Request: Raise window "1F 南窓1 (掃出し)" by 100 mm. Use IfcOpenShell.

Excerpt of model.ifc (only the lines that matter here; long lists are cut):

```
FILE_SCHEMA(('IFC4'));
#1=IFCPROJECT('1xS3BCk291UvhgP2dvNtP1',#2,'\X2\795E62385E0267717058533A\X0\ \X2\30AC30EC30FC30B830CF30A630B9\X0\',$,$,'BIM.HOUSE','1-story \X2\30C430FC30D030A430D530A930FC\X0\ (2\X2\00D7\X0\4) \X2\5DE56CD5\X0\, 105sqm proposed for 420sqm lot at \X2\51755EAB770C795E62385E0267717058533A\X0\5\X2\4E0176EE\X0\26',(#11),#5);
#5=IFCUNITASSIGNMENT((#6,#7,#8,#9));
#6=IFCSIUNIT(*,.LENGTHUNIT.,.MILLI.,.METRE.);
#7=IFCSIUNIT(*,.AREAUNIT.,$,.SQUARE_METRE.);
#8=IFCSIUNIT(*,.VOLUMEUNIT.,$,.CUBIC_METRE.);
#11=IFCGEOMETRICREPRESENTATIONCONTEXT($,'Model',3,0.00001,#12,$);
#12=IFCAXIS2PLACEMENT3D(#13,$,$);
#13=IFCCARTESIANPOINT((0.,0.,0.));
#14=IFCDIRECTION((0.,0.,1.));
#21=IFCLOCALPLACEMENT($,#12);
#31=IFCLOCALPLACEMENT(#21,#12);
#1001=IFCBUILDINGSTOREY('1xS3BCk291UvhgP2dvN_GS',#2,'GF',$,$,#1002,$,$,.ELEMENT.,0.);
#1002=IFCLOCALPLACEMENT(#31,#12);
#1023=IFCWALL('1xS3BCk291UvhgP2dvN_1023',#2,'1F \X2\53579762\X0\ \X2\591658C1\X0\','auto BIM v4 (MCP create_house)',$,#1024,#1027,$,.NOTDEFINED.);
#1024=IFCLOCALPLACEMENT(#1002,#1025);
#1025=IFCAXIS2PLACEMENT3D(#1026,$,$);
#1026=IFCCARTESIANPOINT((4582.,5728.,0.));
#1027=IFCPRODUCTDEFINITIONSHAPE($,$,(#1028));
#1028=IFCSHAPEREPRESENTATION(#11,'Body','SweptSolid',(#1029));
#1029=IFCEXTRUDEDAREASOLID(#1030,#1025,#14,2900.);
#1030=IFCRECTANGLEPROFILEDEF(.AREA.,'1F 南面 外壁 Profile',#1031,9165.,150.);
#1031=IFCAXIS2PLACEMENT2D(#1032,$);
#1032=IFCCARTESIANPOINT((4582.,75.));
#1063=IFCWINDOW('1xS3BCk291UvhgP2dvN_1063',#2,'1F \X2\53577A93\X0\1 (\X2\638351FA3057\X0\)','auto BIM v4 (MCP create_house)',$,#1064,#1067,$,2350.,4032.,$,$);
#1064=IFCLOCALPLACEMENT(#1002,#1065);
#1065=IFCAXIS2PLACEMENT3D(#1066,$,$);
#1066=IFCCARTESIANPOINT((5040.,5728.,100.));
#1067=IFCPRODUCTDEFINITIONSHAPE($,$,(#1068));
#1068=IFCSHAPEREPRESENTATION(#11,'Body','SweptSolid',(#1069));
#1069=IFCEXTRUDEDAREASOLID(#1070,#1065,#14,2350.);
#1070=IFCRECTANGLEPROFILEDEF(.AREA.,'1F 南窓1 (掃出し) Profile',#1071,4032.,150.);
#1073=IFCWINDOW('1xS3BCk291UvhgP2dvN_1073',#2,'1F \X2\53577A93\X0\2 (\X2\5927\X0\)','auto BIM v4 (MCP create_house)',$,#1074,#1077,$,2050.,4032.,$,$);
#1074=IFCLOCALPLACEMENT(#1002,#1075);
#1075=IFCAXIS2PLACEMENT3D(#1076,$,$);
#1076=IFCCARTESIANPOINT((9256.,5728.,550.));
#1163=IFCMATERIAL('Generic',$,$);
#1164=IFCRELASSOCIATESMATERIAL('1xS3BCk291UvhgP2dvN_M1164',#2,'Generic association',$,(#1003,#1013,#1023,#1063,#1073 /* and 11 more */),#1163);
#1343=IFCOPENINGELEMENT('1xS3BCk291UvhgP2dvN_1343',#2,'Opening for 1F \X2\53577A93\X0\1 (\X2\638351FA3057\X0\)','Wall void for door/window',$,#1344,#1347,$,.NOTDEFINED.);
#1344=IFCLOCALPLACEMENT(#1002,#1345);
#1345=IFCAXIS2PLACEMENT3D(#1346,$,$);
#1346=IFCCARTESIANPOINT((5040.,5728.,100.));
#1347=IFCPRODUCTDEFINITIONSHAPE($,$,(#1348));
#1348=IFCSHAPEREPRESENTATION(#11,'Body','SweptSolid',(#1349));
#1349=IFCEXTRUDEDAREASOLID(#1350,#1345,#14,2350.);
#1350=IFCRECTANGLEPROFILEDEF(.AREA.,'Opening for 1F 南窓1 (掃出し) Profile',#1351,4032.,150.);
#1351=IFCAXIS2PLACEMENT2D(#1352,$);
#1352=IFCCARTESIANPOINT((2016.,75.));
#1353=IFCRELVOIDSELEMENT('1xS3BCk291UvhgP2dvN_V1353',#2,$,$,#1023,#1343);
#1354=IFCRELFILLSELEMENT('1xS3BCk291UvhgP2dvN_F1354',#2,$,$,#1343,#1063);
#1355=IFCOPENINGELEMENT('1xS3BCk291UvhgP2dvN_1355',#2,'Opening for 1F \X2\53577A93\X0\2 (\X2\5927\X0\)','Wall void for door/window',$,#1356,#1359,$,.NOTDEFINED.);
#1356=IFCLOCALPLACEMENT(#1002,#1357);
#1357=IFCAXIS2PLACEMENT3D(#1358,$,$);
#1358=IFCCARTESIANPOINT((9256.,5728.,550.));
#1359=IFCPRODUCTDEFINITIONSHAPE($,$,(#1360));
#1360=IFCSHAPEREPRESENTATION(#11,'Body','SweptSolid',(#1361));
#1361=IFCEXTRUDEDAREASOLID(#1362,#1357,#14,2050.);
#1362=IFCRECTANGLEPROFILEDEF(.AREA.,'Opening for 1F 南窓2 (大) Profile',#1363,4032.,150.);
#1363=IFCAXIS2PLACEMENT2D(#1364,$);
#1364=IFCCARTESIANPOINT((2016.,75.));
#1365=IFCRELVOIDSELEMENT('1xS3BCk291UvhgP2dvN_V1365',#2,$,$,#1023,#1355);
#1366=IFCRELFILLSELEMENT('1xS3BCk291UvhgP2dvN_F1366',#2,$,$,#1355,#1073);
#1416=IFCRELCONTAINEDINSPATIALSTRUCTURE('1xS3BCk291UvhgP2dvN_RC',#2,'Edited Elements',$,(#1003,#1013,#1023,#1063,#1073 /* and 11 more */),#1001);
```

```python
import numpy as np
import ifcopenshell
import ifcopenshell.api.geometry
import ifcopenshell.util.placement
import ifcopenshell.util.unit

model = ifcopenshell.open("model.ifc")
unit_scale = ifcopenshell.util.unit.calculate_unit_scale(model)

window = model.by_guid("1xS3BCk291UvhgP2dvN_1063")
opening = window.FillsVoids[0].RelatingOpeningElement
dz = 0.1 / unit_scale

shift = np.array([0.0, 0.0, dz])
# The window is not placed relative to its opening, so move both.
for product in (opening, window):
    matrix = ifcopenshell.util.placement.get_local_placement(product.ObjectPlacement)
    matrix[:3, 3] += shift
    ifcopenshell.api.geometry.edit_object_placement(model, product=product, matrix=matrix, is_si=False)

print(f"moved by {dz * unit_scale:+.3f} m")

model.write("model_v2.ifc")
```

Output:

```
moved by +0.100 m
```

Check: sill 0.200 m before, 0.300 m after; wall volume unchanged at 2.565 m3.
